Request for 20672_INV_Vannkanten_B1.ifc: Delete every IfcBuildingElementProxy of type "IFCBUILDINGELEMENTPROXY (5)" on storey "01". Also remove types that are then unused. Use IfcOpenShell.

First a look at what the model holds.

```python
import ifcopenshell
import ifcopenshell.util.element

model = ifcopenshell.open("20672_INV_Vannkanten_B1.ifc")
print(model.schema)
storey = next(s for s in model.by_type("IfcBuildingStorey") if s.Name == "01")
proxies = [e for e in ifcopenshell.util.element.get_decomposition(storey) if e.is_a("IfcBuildingElementProxy")]
seen = {}
for e in proxies:
    element_type = ifcopenshell.util.element.get_type(e)
    name = element_type.Name if element_type not in (None, e) else None
    seen[name] = seen.get(name, 0) + 1
for name, count in sorted(seen.items(), key=str):
    print(count, "x", name)
```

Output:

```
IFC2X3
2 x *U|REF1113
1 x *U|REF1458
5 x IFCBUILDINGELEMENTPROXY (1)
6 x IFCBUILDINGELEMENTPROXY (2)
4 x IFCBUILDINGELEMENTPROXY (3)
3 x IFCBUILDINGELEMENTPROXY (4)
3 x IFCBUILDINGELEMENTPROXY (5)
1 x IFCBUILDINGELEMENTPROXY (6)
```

```python
import ifcopenshell
import ifcopenshell.api.root
import ifcopenshell.util.element

model = ifcopenshell.open("20672_INV_Vannkanten_B1.ifc")

storey = next(s for s in model.by_type("IfcBuildingStorey") if s.Name == "01")
proxies = [e for e in ifcopenshell.util.element.get_decomposition(storey) if e.is_a("IfcBuildingElementProxy")]
targets = [e for e in proxies if (t := ifcopenshell.util.element.get_type(e)) not in (None, e) and t.Name == "IFCBUILDINGELEMENTPROXY (5)"]
types = {ifcopenshell.util.element.get_type(e) for e in targets} - {None, *targets}

for e in targets:
    ifcopenshell.api.root.remove_product(model, product=e)
print(len(targets), "removed")

unused = [t for t in types if not ifcopenshell.util.element.get_types(t)]
for t in unused:
    ifcopenshell.api.root.remove_product(model, product=t)
print(len(unused), "unused types removed")

model.write("20672_INV_Vannkanten_B1_v2.ifc")
```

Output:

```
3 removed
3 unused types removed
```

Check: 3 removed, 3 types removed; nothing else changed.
